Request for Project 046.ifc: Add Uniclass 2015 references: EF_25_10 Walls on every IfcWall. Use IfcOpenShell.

First a look at what the model holds.

```python
import ifcopenshell

model = ifcopenshell.open("Project 046.ifc")
print(model.schema)
print("classifications:", [c.Name for c in model.by_type("IfcClassification")])
for ifc_class in ("IfcDoor", "IfcRoof", "IfcStair", "IfcWall", "IfcWindow"):
    print(ifc_class, len(model.by_type(ifc_class)))
```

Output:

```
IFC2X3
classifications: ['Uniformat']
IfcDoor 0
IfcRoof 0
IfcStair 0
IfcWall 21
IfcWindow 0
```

```python
import ifcopenshell
import ifcopenshell.api.classification

model = ifcopenshell.open("Project 046.ifc")

# IFC2X3 requires Source and Edition and has no link from the project to the system.
system = model.create_entity("IfcClassification", Source="NBS", Edition="2015", Name="Uniclass 2015")

codes = {
    "IfcWall": ("EF_25_10", "Walls"),
}
for ifc_class, (code, name) in codes.items():
    products = model.by_type(ifc_class)
    ifcopenshell.api.classification.add_reference(
        model, products=products, classification=system, identification=code, name=name
    )
    print(code, len(products))

model.write("Project 046-out.ifc")
```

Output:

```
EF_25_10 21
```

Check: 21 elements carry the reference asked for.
